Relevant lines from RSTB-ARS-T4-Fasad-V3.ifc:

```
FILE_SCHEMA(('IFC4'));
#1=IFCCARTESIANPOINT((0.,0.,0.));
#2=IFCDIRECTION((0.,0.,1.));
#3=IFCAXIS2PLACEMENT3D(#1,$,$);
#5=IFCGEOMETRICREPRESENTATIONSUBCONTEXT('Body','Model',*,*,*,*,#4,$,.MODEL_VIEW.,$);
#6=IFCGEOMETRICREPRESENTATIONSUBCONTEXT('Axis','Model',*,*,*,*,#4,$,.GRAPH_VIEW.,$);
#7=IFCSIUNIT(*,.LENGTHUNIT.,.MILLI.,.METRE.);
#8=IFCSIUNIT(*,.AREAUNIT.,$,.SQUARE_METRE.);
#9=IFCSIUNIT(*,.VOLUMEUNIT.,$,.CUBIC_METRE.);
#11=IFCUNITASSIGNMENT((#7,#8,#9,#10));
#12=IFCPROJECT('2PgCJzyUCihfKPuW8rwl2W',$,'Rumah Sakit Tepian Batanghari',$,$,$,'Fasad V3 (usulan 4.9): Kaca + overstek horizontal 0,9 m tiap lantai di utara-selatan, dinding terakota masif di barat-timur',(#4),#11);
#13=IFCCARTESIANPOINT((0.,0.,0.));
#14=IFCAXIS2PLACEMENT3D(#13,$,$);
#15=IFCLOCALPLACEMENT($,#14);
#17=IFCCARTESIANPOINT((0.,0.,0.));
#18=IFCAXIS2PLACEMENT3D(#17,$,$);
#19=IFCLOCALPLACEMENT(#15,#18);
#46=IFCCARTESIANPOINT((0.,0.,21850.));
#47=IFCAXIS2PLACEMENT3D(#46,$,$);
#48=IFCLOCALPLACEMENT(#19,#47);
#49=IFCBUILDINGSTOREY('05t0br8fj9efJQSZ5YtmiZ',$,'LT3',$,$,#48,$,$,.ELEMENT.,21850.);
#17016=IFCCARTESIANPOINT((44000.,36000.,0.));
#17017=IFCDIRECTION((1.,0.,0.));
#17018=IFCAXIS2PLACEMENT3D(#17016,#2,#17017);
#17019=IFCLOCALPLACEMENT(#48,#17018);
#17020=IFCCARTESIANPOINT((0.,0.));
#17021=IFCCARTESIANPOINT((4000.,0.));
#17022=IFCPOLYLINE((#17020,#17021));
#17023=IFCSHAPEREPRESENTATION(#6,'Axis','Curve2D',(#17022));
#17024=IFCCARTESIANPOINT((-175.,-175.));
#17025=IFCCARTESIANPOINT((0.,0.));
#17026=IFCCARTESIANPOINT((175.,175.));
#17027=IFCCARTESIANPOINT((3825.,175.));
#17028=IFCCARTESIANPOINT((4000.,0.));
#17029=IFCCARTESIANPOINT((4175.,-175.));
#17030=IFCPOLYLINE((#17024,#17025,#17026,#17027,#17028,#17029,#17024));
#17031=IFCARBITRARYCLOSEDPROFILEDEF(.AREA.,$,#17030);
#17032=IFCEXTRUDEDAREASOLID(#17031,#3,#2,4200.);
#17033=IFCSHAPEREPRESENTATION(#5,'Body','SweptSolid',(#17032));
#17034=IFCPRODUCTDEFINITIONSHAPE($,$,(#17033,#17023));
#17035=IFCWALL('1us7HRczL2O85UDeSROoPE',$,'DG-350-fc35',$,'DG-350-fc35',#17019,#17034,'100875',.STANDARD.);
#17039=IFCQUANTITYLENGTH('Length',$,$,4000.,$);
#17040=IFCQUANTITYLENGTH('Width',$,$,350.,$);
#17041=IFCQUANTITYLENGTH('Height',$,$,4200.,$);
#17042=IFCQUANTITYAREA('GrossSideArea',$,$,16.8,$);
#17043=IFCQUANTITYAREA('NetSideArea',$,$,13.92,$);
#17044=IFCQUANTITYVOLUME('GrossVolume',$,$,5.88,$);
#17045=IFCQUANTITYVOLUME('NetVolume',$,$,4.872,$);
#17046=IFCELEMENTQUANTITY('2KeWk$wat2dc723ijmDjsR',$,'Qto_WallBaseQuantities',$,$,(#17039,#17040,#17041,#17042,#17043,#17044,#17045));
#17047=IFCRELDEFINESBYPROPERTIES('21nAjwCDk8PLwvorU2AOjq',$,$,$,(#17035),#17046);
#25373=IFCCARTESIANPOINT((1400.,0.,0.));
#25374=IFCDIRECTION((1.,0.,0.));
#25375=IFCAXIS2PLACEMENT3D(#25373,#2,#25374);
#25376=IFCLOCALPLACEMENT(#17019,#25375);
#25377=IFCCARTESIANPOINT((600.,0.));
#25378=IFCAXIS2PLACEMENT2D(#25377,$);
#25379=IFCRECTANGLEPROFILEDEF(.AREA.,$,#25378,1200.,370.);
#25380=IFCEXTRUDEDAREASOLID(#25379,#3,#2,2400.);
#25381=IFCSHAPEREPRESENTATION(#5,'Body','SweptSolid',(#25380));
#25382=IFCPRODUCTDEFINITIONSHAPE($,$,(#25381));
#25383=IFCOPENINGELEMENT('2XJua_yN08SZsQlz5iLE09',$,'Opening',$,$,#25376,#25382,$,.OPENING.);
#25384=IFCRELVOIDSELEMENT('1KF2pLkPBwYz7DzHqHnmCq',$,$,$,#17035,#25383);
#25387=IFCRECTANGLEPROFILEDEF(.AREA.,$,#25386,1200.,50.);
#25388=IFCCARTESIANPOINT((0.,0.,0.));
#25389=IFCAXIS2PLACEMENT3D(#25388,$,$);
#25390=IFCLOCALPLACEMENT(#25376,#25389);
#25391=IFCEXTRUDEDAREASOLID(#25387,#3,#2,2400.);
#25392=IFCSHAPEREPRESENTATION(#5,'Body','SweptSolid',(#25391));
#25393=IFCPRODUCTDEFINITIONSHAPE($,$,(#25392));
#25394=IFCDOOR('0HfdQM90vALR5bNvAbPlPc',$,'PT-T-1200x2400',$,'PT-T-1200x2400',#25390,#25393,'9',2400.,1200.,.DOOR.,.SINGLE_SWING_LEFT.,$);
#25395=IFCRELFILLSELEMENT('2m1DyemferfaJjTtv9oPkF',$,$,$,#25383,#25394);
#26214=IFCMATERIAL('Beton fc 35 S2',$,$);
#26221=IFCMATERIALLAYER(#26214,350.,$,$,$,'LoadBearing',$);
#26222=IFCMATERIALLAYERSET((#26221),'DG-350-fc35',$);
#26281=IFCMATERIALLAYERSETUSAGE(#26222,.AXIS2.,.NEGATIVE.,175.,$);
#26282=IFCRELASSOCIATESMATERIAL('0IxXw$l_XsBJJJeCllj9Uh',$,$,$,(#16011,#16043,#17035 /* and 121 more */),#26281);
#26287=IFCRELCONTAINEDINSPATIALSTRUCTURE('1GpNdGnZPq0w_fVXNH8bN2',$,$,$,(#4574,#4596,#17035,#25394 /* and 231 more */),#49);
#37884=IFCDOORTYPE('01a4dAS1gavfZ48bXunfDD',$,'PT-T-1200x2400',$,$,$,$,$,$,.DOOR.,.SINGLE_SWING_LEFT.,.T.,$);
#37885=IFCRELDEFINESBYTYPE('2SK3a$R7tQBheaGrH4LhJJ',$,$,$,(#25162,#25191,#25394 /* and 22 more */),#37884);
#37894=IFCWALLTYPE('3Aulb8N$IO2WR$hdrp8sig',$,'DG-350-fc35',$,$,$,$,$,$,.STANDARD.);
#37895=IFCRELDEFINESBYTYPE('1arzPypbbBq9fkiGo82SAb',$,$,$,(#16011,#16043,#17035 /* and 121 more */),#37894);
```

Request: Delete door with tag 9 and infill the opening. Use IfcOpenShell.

```python
import ifcopenshell
import ifcopenshell.api.feature
import ifcopenshell.api.pset
import ifcopenshell.api.root
import ifcopenshell.geom
import ifcopenshell.util.element
import ifcopenshell.util.shape
import ifcopenshell.util.unit

model = ifcopenshell.open("RSTB-ARS-T4-Fasad-V3.ifc")
area_scale = ifcopenshell.util.unit.calculate_unit_scale(model, "AREAUNIT")
volume_scale = ifcopenshell.util.unit.calculate_unit_scale(model, "VOLUMEUNIT")
settings = ifcopenshell.geom.settings()


def volume(element):
    """Net volume in cubic metres, openings subtracted."""
    shape = ifcopenshell.geom.create_shape(settings, element)
    return ifcopenshell.util.shape.get_volume(shape.geometry)


door = model.by_guid("0HfdQM90vALR5bNvAbPlPc")
opening = door.FillsVoids[0].RelatingOpeningElement
wall = opening.VoidsElements[0].RelatingBuildingElement
before = volume(wall)

ifcopenshell.api.root.remove_product(model, product=door)
ifcopenshell.api.feature.remove_feature(model, feature=opening)

after = volume(wall)
thickness = 0.35  # wall thickness in metres

# Update the wall's stored quantities.
qto = model.by_id(ifcopenshell.util.element.get_pset(wall, "Qto_WallBaseQuantities", should_inherit=False)["id"])
ifcopenshell.api.pset.edit_qto(model, qto=qto, properties={
    "NetSideArea": after / thickness / area_scale,
    "NetVolume": after / volume_scale,
})

print(f"wall volume {before:.3f} -> {after:.3f} m3")

model.write("RSTB-ARS-T4-Fasad-V3_v2.ifc")
```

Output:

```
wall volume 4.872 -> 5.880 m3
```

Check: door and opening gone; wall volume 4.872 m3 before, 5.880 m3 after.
